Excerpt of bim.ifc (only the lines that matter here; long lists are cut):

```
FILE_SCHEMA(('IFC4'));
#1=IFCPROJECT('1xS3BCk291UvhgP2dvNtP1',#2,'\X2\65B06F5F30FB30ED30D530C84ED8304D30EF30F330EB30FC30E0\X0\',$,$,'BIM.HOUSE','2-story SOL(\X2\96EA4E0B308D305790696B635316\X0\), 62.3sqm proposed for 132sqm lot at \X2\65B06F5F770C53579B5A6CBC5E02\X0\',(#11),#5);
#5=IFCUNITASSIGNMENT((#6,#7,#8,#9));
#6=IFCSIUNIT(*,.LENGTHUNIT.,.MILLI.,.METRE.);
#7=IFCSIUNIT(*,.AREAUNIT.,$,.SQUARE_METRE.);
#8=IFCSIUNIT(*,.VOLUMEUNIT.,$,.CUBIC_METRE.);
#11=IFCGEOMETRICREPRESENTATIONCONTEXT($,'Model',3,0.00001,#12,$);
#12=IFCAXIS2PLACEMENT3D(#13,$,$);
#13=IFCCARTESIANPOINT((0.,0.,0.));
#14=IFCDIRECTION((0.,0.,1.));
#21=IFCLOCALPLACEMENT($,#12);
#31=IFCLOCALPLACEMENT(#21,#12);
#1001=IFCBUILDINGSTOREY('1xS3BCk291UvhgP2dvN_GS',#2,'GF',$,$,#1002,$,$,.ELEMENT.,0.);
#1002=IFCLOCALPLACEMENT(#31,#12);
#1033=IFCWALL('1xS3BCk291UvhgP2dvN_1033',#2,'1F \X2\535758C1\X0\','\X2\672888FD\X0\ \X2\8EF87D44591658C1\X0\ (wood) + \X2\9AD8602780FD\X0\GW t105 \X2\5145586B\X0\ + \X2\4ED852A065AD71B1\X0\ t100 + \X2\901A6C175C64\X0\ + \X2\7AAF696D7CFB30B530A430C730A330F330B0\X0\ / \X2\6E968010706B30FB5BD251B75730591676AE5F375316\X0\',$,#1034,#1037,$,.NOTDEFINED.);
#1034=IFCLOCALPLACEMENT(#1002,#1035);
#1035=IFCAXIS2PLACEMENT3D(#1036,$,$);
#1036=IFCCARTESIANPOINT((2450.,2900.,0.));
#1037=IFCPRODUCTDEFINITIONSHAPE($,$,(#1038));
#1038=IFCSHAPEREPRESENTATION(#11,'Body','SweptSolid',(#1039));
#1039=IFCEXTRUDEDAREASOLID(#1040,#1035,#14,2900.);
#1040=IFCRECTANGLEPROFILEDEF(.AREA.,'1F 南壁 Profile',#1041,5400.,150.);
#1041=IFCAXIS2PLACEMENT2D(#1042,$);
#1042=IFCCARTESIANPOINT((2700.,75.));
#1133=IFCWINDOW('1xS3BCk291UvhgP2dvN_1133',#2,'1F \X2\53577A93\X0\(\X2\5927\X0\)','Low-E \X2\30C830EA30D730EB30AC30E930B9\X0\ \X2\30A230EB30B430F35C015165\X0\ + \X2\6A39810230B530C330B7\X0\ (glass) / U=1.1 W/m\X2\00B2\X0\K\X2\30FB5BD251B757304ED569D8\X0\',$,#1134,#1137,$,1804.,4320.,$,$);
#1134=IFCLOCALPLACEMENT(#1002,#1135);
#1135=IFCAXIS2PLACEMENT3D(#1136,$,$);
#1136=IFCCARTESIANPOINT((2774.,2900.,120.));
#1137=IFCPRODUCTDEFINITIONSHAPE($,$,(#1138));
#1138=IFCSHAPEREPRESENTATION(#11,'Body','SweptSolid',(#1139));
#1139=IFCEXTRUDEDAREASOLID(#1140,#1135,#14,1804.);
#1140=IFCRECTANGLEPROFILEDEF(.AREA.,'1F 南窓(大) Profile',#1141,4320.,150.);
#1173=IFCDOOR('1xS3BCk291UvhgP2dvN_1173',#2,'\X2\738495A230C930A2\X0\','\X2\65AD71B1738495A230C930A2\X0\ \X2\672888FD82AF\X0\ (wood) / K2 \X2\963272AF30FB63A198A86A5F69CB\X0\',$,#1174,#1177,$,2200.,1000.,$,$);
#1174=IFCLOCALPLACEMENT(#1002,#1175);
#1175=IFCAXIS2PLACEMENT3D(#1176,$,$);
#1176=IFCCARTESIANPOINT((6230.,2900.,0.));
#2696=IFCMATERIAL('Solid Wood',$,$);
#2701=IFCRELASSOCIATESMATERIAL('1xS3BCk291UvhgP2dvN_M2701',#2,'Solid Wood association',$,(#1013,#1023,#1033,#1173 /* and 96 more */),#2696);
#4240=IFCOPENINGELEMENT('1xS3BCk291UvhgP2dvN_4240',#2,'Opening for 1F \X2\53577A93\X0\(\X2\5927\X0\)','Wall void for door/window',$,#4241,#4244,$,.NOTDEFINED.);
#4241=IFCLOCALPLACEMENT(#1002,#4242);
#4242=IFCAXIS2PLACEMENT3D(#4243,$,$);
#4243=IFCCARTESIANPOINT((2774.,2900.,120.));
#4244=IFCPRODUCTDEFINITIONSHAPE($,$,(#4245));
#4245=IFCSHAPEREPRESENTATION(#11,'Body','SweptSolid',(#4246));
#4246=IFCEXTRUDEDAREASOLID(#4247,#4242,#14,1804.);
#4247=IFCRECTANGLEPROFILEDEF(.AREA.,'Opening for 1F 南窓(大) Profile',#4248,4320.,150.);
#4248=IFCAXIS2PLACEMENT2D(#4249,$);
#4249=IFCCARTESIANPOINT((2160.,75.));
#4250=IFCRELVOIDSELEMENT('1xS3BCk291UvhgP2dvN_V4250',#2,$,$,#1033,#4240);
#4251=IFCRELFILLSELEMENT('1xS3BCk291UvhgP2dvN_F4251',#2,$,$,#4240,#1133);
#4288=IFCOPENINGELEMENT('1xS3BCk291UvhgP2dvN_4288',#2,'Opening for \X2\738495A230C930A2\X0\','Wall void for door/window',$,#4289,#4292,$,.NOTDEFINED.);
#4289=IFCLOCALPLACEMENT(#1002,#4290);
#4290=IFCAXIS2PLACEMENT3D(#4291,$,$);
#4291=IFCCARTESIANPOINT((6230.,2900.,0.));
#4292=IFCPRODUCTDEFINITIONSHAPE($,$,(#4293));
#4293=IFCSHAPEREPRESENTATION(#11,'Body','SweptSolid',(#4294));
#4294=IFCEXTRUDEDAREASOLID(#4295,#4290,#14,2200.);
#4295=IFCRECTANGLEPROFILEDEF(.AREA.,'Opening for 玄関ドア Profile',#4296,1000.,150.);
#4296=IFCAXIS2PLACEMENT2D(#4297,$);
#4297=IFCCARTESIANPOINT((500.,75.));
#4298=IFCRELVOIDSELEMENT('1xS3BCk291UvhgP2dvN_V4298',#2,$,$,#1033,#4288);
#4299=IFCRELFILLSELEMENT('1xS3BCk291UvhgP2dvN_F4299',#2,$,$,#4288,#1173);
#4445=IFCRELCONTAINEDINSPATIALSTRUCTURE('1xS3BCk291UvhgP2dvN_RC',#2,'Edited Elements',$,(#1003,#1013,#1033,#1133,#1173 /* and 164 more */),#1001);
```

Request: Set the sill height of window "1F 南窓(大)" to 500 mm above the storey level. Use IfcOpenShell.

```python
import numpy as np
import ifcopenshell
import ifcopenshell.api.geometry
import ifcopenshell.geom
import ifcopenshell.util.element
import ifcopenshell.util.placement
import ifcopenshell.util.shape
import ifcopenshell.util.unit

model = ifcopenshell.open("bim.ifc")
unit_scale = ifcopenshell.util.unit.calculate_unit_scale(model)

window = model.by_id(1133)
opening = window.FillsVoids[0].RelatingOpeningElement
storey = ifcopenshell.util.element.get_container(window, ifc_class="IfcBuildingStorey")
level = ifcopenshell.util.placement.get_local_placement(storey.ObjectPlacement)[2, 3]

# The opening's origin need not be at the sill, so measure its lowest point.
shape = ifcopenshell.geom.create_shape(ifcopenshell.geom.settings(), opening)
bottom = ifcopenshell.util.shape.get_shape_bottom_elevation(shape, shape.geometry) / unit_scale
dz = level + 500.0 - bottom

shift = np.array([0.0, 0.0, dz])
# The window is not placed relative to its opening, so move both.
for product in (opening, window):
    matrix = ifcopenshell.util.placement.get_local_placement(product.ObjectPlacement)
    matrix[:3, 3] += shift
    ifcopenshell.api.geometry.edit_object_placement(model, product=product, matrix=matrix, is_si=False)

print(f"moved by {dz * unit_scale:+.3f} m")

model.write("bim-out.ifc")
```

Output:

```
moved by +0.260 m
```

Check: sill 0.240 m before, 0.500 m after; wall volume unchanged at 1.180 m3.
